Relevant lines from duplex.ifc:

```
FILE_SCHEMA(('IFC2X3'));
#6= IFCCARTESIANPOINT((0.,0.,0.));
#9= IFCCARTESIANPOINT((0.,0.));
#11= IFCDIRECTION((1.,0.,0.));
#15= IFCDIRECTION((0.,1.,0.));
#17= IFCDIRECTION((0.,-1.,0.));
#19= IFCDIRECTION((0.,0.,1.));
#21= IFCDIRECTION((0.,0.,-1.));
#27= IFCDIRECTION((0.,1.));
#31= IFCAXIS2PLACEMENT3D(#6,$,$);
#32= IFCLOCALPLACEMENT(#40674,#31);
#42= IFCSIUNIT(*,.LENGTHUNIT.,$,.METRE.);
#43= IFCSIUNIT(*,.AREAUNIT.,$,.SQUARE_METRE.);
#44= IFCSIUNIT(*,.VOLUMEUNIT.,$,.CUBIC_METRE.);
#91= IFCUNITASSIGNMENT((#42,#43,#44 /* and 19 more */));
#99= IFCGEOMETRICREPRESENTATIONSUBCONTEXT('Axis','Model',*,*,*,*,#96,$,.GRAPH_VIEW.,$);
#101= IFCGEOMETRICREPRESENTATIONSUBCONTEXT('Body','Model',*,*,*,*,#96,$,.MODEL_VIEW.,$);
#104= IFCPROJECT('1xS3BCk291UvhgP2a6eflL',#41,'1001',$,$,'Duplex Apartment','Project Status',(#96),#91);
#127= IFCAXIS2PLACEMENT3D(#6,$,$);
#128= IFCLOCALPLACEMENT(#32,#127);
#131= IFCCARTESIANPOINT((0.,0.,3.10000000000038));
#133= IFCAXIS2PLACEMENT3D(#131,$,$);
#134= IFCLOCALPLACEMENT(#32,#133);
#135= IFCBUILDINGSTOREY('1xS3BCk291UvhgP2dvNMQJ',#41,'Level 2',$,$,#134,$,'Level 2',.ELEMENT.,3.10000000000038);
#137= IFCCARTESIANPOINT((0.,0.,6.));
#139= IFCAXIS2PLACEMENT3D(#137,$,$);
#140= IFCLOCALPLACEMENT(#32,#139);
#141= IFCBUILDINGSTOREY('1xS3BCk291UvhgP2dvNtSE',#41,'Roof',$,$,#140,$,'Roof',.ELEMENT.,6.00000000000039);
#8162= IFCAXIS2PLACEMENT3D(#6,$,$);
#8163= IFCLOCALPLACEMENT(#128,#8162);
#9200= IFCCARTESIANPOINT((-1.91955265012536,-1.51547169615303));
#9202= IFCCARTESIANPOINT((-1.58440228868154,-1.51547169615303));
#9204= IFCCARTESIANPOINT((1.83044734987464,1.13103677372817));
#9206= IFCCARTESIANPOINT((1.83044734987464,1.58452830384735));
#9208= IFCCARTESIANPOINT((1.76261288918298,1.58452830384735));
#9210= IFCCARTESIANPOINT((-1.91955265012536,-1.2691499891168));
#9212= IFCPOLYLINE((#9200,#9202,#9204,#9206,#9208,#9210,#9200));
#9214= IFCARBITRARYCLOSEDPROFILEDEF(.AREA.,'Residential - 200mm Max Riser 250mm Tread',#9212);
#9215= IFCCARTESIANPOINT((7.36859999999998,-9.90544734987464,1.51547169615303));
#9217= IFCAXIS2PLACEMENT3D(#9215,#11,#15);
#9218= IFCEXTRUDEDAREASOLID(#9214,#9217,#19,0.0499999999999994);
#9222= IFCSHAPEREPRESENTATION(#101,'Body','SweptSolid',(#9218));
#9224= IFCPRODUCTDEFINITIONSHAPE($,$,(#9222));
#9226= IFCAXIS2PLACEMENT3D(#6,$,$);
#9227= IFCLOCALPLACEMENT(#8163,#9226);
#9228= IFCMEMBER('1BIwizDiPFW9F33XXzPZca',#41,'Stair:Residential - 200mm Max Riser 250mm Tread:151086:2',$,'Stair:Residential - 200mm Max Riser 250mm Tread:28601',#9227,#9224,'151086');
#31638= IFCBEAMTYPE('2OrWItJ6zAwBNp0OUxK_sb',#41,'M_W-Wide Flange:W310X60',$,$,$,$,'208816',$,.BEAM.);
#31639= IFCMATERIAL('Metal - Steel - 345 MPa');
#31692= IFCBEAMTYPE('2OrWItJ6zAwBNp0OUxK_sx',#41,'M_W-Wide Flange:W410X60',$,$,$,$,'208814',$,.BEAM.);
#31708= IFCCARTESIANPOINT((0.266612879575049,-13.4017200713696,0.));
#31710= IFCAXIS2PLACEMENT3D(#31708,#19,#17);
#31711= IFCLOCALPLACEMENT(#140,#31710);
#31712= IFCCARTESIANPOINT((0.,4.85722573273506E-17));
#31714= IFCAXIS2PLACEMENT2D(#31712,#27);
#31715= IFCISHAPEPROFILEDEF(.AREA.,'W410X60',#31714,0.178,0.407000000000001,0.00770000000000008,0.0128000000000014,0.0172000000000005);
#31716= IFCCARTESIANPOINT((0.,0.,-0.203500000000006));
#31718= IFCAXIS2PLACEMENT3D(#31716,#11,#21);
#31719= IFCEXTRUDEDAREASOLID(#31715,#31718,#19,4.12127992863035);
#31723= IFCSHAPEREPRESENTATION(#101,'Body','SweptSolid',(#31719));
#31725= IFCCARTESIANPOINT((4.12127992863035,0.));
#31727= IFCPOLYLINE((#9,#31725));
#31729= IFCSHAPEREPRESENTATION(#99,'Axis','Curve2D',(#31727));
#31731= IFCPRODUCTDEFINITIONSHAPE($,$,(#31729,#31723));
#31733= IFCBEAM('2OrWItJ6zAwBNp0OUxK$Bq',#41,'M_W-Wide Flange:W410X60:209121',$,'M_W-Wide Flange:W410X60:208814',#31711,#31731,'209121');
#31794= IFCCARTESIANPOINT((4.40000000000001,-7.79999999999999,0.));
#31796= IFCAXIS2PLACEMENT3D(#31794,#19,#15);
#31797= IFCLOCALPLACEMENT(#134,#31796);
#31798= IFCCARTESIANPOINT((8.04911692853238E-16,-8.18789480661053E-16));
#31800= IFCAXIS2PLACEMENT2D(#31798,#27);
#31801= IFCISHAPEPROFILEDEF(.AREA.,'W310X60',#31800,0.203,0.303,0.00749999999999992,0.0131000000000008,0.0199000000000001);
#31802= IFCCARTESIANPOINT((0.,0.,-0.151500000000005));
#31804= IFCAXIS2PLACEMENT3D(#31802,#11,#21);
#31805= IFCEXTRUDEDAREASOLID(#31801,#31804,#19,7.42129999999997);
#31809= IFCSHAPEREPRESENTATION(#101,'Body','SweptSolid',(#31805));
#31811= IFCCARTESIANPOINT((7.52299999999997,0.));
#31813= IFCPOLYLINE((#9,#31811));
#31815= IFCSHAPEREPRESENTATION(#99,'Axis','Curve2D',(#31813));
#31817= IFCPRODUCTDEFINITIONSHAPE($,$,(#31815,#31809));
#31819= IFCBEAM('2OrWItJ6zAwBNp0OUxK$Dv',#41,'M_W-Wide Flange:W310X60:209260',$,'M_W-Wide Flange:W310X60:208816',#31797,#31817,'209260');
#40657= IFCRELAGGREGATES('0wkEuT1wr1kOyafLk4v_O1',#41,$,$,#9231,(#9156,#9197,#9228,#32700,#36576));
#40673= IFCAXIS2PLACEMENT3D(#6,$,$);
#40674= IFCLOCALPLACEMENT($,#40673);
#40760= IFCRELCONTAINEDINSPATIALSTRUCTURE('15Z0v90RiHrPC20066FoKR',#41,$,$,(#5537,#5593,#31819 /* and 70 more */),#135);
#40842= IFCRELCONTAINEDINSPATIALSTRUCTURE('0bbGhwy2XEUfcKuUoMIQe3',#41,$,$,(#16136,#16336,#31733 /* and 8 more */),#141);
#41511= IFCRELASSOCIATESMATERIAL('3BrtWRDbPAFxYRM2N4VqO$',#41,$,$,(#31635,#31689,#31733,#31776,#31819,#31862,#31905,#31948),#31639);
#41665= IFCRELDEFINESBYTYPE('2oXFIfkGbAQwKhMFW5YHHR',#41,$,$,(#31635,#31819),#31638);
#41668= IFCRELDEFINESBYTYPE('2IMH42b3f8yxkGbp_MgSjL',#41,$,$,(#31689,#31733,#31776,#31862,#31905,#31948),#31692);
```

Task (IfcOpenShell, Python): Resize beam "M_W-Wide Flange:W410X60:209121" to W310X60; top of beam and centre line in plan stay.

```python
import ifcopenshell
import ifcopenshell.api.type
import ifcopenshell.util.element
import ifcopenshell.util.representation

model = ifcopenshell.open("duplex.ifc")

member = model.by_guid("2OrWItJ6zAwBNp0OUxK$Bq")
source = next(p for p in model.by_type("IfcIShapeProfileDef") if p.ProfileName == "W310X60")

body = ifcopenshell.util.representation.get_representation(member, "Model", "Body")
solid = body.Items[0]
old_profile = solid.SweptArea

# Copy the section's sizes but keep this member's own profile position.
profile = ifcopenshell.util.element.copy(model, source)
# Profiles are centred, so shift by half the change in depth to hold the top.
shift = (old_profile.OverallDepth - profile.OverallDepth) / 2
x, y = old_profile.Position.Location.Coordinates
up = (-1.0, 0.0)  # upwards, in the solid's own plane
location = model.createIfcCartesianPoint((x + up[0] * shift, y + up[1] * shift))
profile.Position = model.createIfcAxis2Placement2D(location, old_profile.Position.RefDirection)
solid.SweptArea = profile
if not model.get_total_inverses(old_profile):
    ifcopenshell.util.element.remove_deep2(model, old_profile)

new_type = model.by_id(31638)
ifcopenshell.api.type.assign_type(
    model, related_objects=[member], relating_type=new_type, should_map_representations=False
)
member.Name = member.Name.replace("W410X60", "W310X60")
member.ObjectType = "M_W-Wide Flange:W310X60:208814"

print(solid.SweptArea)

model.write("duplex_updated.ifc")
```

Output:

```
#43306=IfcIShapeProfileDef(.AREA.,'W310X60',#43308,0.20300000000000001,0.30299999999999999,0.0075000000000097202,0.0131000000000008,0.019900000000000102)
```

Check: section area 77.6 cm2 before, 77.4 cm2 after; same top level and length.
